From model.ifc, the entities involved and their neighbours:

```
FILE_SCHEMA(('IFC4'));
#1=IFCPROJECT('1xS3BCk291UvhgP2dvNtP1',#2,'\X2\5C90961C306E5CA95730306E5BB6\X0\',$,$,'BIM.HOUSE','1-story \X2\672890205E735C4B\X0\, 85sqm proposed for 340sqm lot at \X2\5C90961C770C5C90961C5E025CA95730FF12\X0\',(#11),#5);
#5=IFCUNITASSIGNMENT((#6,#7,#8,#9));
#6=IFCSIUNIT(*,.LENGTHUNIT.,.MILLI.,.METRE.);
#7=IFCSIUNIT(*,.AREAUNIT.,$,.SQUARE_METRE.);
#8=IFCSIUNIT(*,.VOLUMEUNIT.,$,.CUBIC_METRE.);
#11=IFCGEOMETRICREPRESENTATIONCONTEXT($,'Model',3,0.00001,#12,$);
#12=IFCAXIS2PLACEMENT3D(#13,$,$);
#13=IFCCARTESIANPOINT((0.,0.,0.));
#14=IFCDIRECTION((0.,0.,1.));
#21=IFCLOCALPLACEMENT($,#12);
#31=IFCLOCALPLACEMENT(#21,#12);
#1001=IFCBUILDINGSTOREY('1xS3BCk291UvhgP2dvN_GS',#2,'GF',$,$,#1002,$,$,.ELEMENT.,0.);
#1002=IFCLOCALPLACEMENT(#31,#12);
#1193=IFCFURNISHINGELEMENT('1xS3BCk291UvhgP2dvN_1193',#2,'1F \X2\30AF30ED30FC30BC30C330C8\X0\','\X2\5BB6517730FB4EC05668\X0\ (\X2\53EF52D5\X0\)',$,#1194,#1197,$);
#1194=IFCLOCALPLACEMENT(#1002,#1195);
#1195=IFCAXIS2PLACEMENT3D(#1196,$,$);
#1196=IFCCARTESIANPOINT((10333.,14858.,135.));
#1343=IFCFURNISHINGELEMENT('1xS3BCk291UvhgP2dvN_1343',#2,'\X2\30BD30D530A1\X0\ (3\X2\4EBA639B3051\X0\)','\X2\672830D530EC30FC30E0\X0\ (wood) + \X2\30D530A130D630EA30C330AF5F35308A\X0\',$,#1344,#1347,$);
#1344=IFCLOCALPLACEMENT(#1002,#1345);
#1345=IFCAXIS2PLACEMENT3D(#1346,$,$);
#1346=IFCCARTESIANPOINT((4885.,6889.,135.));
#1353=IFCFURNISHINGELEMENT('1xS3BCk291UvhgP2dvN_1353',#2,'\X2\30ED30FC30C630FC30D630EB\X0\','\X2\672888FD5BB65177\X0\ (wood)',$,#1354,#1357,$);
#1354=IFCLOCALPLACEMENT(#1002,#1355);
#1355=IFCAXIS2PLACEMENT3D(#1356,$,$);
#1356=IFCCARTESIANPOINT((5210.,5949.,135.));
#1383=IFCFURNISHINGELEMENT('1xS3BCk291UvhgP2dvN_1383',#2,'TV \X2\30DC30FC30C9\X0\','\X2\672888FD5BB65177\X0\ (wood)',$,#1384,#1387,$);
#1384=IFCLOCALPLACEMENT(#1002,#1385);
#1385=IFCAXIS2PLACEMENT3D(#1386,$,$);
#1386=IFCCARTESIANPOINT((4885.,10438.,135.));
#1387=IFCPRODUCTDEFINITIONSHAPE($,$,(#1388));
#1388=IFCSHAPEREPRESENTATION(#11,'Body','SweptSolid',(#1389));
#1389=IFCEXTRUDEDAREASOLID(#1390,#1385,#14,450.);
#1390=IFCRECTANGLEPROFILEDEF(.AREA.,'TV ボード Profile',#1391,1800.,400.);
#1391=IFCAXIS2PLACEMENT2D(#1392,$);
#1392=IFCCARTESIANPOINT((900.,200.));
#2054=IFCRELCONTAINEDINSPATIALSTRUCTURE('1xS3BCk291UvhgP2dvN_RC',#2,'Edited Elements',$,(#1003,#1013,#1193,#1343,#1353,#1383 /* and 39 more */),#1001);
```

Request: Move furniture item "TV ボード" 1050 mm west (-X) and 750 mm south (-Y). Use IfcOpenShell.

```python
import ifcopenshell
import ifcopenshell.api.geometry
import ifcopenshell.util.placement
import ifcopenshell.util.unit

model = ifcopenshell.open("model.ifc")
unit_scale = ifcopenshell.util.unit.calculate_unit_scale(model)

item = model.by_guid("1xS3BCk291UvhgP2dvN_1383")
matrix = ifcopenshell.util.placement.get_local_placement(item.ObjectPlacement)
matrix[0, 3] -= 1.05 / unit_scale
matrix[1, 3] -= 0.75 / unit_scale
ifcopenshell.api.geometry.edit_object_placement(model, product=item, matrix=matrix, is_si=False)

print(ifcopenshell.util.placement.get_local_placement(item.ObjectPlacement).round(3) + 0.0)

model.write("model_updated.ifc")
```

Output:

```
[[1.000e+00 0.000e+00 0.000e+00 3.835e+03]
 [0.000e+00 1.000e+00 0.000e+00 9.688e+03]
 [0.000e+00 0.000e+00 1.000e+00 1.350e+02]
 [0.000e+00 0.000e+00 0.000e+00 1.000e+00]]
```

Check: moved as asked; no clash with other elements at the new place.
